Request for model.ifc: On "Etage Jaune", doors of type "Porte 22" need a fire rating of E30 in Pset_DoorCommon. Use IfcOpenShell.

First a look at what the model holds.

```python
import ifcopenshell
import ifcopenshell.util.element

model = ifcopenshell.open("model.ifc")
print(model.schema)
storey = next(s for s in model.by_type("IfcBuildingStorey") if s.Name == "Etage Jaune")
doors = [e for e in ifcopenshell.util.element.get_decomposition(storey) if e.is_a("IfcDoor")]
seen = {}
for e in doors:
    element_type = ifcopenshell.util.element.get_type(e)
    key = (element_type.Name if element_type != e and element_type else None, ifcopenshell.util.element.get_pset(e, "Pset_DoorCommon", "FireRating"))
    seen[key] = seen.get(key, 0) + 1
for (name, value), count in sorted(seen.items(), key=str):
    print(count, "x", name, "|", value)
```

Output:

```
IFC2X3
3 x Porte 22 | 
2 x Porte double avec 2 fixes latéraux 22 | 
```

```python
import ifcopenshell
import ifcopenshell.api.pset
import ifcopenshell.util.element

model = ifcopenshell.open("model.ifc")

storey = next(s for s in model.by_type("IfcBuildingStorey") if s.Name == "Etage Jaune")
doors = [e for e in ifcopenshell.util.element.get_decomposition(storey) if e.is_a("IfcDoor")]

count = 0
for e in doors:
    element_type = ifcopenshell.util.element.get_type(e)
    if element_type in (None, e) or element_type.Name != "Porte 22":
        continue
    # add_pset returns the element's existing set when there is one.
    pset = ifcopenshell.api.pset.add_pset(model, product=e, name="Pset_DoorCommon")
    ifcopenshell.api.pset.edit_pset(model, pset=pset, properties={"FireRating": "E30"})
    count += 1

print(count, "doors updated")

model.write("model-out.ifc")
```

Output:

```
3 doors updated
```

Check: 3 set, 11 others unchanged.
